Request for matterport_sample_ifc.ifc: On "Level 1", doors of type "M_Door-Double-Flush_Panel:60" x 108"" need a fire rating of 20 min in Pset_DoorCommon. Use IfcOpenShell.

First a look at what the model holds.

```python
import ifcopenshell
import ifcopenshell.util.element

model = ifcopenshell.open("matterport_sample_ifc.ifc")
print(model.schema)
storey = next(s for s in model.by_type("IfcBuildingStorey") if s.Name == "Level 1")
doors = [e for e in ifcopenshell.util.element.get_decomposition(storey) if e.is_a("IfcDoor")]
seen = {}
for e in doors:
    element_type = ifcopenshell.util.element.get_type(e)
    key = (element_type.Name if element_type != e and element_type else None, ifcopenshell.util.element.get_pset(e, "Pset_DoorCommon", "FireRating"))
    seen[key] = seen.get(key, 0) + 1
for (name, value), count in sorted(seen.items(), key=str):
    print(count, "x", name, "|", value)
```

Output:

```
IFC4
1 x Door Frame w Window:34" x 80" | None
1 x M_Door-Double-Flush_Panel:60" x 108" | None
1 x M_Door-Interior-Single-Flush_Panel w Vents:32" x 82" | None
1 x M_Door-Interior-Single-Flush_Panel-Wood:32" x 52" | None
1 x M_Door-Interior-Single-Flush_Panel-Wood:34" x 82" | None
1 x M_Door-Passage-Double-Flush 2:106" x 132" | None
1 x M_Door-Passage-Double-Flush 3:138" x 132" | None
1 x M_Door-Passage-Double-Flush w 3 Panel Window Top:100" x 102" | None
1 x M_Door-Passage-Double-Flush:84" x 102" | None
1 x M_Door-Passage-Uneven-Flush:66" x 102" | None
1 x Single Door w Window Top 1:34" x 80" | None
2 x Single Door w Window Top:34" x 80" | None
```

```python
import ifcopenshell
import ifcopenshell.api.pset
import ifcopenshell.util.element

model = ifcopenshell.open("matterport_sample_ifc.ifc")

storey = next(s for s in model.by_type("IfcBuildingStorey") if s.Name == "Level 1")
doors = [e for e in ifcopenshell.util.element.get_decomposition(storey) if e.is_a("IfcDoor")]

count = 0
for e in doors:
    element_type = ifcopenshell.util.element.get_type(e)
    if element_type in (None, e) or element_type.Name != 'M_Door-Double-Flush_Panel:60" x 108"':
        continue
    # add_pset returns the element's existing set when there is one.
    pset = ifcopenshell.api.pset.add_pset(model, product=e, name="Pset_DoorCommon")
    ifcopenshell.api.pset.edit_pset(model, pset=pset, properties={"FireRating": "20 min"})
    count += 1

print(count, "doors updated")

model.write("matterport_sample_ifc-out.ifc")
```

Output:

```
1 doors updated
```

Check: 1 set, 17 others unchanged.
